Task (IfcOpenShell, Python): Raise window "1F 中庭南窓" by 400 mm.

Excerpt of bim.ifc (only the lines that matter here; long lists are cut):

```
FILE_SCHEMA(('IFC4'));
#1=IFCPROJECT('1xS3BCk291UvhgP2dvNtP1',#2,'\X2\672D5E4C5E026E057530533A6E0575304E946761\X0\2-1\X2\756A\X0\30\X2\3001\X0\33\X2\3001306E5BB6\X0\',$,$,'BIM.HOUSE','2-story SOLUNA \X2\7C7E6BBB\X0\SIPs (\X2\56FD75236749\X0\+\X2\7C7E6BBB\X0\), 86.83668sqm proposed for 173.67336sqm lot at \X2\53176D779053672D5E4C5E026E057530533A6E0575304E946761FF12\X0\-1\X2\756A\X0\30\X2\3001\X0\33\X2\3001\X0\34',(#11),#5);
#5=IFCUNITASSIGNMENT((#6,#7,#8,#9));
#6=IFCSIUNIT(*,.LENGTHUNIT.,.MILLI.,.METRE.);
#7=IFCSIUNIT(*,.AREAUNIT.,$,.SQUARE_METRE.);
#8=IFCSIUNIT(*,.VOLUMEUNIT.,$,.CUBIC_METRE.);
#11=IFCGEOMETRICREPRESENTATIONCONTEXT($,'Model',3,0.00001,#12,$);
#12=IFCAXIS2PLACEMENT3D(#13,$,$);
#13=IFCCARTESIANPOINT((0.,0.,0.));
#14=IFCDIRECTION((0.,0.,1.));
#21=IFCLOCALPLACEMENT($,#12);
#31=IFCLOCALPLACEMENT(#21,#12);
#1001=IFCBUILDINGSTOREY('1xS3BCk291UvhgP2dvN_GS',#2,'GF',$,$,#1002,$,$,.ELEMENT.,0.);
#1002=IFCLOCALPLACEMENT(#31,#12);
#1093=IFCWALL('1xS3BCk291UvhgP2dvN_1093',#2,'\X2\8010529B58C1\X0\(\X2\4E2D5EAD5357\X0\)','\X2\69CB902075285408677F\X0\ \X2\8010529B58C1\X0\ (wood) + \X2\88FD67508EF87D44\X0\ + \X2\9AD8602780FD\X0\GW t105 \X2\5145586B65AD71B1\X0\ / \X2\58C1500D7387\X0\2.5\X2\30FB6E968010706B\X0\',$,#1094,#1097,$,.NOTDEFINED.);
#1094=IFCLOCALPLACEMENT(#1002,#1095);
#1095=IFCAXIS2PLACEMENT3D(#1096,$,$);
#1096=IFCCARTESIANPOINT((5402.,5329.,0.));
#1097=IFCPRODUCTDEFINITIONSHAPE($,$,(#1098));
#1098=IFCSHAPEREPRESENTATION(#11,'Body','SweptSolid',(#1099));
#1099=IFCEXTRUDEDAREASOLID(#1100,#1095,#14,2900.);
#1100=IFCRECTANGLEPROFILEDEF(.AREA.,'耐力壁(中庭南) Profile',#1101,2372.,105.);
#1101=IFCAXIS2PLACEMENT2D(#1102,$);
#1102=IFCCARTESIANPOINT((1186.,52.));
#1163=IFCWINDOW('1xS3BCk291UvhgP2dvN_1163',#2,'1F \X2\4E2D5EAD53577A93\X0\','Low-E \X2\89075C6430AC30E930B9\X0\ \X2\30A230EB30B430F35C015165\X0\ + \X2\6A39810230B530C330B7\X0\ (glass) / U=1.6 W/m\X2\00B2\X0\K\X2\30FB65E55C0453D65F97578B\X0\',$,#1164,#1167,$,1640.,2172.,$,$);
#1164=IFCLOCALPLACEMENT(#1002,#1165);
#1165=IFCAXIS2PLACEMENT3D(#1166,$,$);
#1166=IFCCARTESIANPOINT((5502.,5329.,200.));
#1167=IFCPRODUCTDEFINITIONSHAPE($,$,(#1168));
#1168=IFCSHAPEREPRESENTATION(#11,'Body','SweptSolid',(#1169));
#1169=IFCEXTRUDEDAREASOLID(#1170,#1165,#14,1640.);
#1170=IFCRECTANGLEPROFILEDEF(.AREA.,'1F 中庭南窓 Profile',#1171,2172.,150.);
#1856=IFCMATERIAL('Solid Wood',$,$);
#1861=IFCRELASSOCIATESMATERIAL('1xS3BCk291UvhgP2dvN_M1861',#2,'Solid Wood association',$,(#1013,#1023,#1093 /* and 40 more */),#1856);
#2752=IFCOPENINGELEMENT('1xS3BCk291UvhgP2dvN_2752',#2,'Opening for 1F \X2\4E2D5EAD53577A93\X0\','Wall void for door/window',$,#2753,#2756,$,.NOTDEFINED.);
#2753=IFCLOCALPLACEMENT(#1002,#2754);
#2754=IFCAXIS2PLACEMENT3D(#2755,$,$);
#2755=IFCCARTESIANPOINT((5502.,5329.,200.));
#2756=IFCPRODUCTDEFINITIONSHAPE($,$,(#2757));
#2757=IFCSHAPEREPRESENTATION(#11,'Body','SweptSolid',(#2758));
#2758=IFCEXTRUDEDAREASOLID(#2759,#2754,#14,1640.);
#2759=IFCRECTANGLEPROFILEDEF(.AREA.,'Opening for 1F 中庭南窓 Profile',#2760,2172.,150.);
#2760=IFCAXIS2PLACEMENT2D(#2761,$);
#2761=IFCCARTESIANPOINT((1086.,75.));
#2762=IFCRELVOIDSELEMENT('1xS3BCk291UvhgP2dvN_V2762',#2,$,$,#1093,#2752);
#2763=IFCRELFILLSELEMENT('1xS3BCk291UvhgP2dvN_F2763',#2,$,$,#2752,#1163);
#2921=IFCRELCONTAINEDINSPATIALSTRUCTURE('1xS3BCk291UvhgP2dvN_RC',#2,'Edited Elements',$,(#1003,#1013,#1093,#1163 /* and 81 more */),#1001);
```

```python
import numpy as np
import ifcopenshell
import ifcopenshell.api.geometry
import ifcopenshell.util.placement
import ifcopenshell.util.unit

model = ifcopenshell.open("bim.ifc")
unit_scale = ifcopenshell.util.unit.calculate_unit_scale(model)

window = model.by_guid("1xS3BCk291UvhgP2dvN_1163")
opening = window.FillsVoids[0].RelatingOpeningElement
dz = 0.4 / unit_scale

shift = np.array([0.0, 0.0, dz])
# The window is not placed relative to its opening, so move both.
for product in (opening, window):
    matrix = ifcopenshell.util.placement.get_local_placement(product.ObjectPlacement)
    matrix[:3, 3] += shift
    ifcopenshell.api.geometry.edit_object_placement(model, product=product, matrix=matrix, is_si=False)

print(f"moved by {dz * unit_scale:+.3f} m")

model.write("bim-out.ifc")
```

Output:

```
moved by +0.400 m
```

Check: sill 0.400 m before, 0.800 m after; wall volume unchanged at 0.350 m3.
